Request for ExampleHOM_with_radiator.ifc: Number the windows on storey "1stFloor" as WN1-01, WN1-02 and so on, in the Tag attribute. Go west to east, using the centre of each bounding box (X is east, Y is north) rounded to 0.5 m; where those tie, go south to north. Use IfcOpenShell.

First a look at what the model holds.

```python
import ifcopenshell
import ifcopenshell.util.element
import ifcopenshell.util.placement

model = ifcopenshell.open("ExampleHOM_with_radiator.ifc")
print(model.schema)
storey = next(s for s in model.by_type("IfcBuildingStorey") if s.Name == "1stFloor")
windows = [e for e in ifcopenshell.util.element.get_decomposition(storey) if e.is_a("IfcWindow")]
for e in sorted(windows, key=lambda e: e.id()):
    origin = ifcopenshell.util.placement.get_local_placement(e.ObjectPlacement)[:3, 3]
    print(e.id(), e.Tag, e.Name, origin.round(2) + 0.0, sep=" | ")
```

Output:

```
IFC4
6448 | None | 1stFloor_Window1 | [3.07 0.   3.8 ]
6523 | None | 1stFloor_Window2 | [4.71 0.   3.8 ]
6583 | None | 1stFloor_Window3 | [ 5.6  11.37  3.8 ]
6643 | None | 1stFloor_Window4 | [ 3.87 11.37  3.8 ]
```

```python
import ifcopenshell
import ifcopenshell.geom
import ifcopenshell.util.element
import ifcopenshell.util.shape

model = ifcopenshell.open("ExampleHOM_with_radiator.ifc")
settings = ifcopenshell.geom.settings()
settings.set("use-world-coords", True)


def centre(element):
    shape = ifcopenshell.geom.create_shape(settings, element)
    return ifcopenshell.util.shape.get_bbox_centroid(shape.geometry)


storey = next(s for s in model.by_type("IfcBuildingStorey") if s.Name == "1stFloor")
windows = [e for e in ifcopenshell.util.element.get_decomposition(storey) if e.is_a("IfcWindow")]

# Insertion points can sit at a corner or the storey origin, so sort by the geometry (in metres).
centres = {e: centre(e) for e in windows}
windows.sort(key=lambda e: (round(centres[e][0] / 0.5), centres[e][1]))

for i, e in enumerate(windows, start=1):
    number = f"WN1-{i:02d}"
    e.Tag = number
    print(e.id(), number)

model.write("ExampleHOM_with_radiator_rev.ifc")
```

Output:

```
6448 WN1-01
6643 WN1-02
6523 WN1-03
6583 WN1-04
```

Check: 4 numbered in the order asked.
